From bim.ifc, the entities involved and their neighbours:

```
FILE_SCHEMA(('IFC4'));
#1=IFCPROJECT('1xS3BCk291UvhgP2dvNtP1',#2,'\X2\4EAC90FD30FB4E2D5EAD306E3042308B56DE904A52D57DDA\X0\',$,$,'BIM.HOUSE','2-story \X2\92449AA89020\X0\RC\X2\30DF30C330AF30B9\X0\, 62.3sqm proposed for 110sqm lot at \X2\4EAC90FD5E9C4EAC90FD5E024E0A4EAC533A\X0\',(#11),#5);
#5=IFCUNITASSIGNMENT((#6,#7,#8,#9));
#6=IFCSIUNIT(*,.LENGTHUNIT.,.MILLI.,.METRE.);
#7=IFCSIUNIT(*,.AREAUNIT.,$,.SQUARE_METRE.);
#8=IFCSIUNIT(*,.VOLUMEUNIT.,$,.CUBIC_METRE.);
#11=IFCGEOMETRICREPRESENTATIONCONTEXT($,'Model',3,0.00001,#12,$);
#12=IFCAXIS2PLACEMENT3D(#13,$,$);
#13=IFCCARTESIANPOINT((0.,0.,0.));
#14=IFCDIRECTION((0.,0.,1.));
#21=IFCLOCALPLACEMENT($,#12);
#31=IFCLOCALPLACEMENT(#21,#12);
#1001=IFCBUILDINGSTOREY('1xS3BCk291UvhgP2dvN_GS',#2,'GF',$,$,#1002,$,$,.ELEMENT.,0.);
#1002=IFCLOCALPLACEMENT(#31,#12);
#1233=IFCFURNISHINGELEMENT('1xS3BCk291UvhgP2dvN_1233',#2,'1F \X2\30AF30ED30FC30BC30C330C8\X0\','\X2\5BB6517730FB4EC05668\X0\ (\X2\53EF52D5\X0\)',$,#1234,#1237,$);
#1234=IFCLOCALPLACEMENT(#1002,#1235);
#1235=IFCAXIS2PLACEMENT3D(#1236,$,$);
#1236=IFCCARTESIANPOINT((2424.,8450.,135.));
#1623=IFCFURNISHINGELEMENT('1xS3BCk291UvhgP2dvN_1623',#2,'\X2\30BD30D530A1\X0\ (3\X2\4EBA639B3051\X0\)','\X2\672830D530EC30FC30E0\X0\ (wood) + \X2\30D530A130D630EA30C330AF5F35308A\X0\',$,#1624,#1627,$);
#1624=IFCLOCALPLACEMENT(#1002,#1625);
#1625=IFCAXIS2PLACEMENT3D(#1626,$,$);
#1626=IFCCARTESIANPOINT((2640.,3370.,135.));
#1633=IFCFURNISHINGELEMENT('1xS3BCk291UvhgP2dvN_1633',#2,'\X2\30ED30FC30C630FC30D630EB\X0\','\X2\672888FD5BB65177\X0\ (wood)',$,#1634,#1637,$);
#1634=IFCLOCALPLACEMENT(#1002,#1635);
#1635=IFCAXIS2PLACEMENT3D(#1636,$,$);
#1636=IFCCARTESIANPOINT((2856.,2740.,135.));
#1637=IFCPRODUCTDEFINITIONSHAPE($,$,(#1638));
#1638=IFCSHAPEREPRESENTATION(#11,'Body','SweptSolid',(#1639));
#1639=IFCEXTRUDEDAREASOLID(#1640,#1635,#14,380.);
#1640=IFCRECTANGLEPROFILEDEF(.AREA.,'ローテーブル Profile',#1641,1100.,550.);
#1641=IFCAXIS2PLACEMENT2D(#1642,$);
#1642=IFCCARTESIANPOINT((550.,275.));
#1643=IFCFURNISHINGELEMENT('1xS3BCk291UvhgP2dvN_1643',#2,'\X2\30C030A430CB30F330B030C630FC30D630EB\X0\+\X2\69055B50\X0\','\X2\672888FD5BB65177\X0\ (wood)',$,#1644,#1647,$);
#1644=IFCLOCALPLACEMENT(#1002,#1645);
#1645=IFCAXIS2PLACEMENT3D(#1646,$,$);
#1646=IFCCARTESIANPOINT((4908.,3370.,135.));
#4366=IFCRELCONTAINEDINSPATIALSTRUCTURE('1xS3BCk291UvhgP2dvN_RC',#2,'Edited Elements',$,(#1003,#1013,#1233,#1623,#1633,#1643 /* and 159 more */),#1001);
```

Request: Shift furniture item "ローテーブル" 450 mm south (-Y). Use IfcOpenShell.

```python
import ifcopenshell
import ifcopenshell.api.geometry
import ifcopenshell.util.placement
import ifcopenshell.util.unit

model = ifcopenshell.open("bim.ifc")
unit_scale = ifcopenshell.util.unit.calculate_unit_scale(model)

item = model.by_id(1633)
matrix = ifcopenshell.util.placement.get_local_placement(item.ObjectPlacement)
matrix[1, 3] -= 0.45 / unit_scale
ifcopenshell.api.geometry.edit_object_placement(model, product=item, matrix=matrix, is_si=False)

print(ifcopenshell.util.placement.get_local_placement(item.ObjectPlacement).round(3) + 0.0)

model.write("bim_updated.ifc")
```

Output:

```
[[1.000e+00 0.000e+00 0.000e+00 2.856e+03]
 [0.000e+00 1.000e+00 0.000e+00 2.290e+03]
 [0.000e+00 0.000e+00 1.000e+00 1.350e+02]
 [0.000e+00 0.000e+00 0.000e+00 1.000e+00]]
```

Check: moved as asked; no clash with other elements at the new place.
